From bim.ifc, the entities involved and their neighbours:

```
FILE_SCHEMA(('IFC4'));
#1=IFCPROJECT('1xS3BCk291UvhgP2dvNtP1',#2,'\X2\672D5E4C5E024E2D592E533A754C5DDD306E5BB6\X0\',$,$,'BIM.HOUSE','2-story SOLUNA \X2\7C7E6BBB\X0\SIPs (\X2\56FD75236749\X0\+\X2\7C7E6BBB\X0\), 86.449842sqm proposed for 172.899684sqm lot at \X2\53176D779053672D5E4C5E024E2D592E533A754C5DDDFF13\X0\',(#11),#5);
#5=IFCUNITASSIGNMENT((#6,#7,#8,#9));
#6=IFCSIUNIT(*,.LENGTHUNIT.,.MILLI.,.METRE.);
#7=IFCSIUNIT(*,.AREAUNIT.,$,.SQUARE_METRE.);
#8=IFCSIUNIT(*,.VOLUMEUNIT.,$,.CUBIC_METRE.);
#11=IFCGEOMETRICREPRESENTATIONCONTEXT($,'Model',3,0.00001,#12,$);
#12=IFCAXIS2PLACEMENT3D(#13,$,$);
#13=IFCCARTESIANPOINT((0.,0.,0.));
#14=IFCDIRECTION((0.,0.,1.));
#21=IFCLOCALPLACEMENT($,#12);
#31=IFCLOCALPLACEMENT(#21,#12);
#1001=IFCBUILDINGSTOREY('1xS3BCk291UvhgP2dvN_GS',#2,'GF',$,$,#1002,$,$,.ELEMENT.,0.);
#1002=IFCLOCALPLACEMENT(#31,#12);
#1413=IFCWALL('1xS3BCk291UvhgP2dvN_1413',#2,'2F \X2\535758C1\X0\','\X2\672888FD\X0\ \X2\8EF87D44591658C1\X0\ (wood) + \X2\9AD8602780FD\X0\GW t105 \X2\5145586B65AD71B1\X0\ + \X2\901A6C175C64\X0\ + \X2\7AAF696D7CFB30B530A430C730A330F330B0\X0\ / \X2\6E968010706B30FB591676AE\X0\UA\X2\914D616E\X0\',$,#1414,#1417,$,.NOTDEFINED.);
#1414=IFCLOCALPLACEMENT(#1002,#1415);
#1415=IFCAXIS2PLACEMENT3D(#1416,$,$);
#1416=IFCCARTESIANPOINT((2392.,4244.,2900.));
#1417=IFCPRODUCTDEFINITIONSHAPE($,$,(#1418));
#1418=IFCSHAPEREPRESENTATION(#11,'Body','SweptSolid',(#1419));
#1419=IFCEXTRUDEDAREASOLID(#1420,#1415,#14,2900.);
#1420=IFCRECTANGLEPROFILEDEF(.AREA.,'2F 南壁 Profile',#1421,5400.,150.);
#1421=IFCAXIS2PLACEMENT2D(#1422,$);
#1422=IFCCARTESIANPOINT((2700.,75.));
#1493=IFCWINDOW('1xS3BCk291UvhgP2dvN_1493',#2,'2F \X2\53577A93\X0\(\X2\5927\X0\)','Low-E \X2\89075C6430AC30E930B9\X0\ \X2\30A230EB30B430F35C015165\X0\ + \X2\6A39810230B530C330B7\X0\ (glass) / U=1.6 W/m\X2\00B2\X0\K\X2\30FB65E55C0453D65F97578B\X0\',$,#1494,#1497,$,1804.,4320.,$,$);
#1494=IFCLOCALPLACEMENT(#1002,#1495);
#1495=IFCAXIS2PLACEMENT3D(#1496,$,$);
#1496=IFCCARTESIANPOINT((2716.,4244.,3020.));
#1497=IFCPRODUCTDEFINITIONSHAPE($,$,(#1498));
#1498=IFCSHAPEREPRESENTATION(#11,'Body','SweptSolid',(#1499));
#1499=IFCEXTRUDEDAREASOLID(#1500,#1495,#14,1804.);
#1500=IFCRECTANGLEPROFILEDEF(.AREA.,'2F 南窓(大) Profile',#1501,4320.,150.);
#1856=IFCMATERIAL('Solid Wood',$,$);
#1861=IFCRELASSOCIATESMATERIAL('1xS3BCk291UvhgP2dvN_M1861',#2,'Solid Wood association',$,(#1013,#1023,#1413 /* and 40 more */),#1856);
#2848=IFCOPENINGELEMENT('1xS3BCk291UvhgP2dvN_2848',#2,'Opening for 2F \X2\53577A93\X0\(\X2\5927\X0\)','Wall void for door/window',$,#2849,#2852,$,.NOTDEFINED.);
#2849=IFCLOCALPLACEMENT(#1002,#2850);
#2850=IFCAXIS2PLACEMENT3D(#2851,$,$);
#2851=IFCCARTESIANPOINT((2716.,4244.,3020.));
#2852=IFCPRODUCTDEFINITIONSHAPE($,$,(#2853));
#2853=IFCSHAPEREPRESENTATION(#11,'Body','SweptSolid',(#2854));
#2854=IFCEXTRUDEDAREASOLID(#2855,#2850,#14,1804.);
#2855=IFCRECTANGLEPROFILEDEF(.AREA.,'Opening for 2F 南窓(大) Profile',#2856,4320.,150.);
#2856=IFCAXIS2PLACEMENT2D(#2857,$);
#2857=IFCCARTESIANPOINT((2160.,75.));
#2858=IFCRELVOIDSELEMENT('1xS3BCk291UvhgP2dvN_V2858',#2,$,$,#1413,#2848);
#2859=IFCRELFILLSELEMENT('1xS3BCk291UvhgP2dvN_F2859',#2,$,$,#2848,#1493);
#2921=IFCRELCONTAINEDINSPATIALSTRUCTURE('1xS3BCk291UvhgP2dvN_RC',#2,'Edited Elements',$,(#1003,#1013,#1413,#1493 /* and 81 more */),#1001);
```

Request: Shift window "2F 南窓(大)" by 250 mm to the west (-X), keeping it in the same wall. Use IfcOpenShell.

```python
import ifcopenshell
import ifcopenshell.api.geometry
import ifcopenshell.util.placement
import ifcopenshell.util.unit

model = ifcopenshell.open("bim.ifc")
unit_scale = ifcopenshell.util.unit.calculate_unit_scale(model)

window = model.by_guid("1xS3BCk291UvhgP2dvN_1493")
opening = window.FillsVoids[0].RelatingOpeningElement
wall = opening.VoidsElements[0].RelatingBuildingElement

wall_matrix = ifcopenshell.util.placement.get_local_placement(wall.ObjectPlacement)
shift = wall_matrix[:3, 0] * -0.25 / unit_scale
before = ifcopenshell.util.placement.get_local_placement(window.ObjectPlacement)[:3, 3].copy()

# The window is not placed relative to its opening, so move both.
for product in (opening, window):
    matrix = ifcopenshell.util.placement.get_local_placement(product.ObjectPlacement)
    matrix[:3, 3] += shift
    ifcopenshell.api.geometry.edit_object_placement(model, product=product, matrix=matrix, is_si=False)

after = ifcopenshell.util.placement.get_local_placement(window.ObjectPlacement)[:3, 3]
print("window moved by", (after - before).round(3) + 0.0)

model.write("bim_edited.ifc")
```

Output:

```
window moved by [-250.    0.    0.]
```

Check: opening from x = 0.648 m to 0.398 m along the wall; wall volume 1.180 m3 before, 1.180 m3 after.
